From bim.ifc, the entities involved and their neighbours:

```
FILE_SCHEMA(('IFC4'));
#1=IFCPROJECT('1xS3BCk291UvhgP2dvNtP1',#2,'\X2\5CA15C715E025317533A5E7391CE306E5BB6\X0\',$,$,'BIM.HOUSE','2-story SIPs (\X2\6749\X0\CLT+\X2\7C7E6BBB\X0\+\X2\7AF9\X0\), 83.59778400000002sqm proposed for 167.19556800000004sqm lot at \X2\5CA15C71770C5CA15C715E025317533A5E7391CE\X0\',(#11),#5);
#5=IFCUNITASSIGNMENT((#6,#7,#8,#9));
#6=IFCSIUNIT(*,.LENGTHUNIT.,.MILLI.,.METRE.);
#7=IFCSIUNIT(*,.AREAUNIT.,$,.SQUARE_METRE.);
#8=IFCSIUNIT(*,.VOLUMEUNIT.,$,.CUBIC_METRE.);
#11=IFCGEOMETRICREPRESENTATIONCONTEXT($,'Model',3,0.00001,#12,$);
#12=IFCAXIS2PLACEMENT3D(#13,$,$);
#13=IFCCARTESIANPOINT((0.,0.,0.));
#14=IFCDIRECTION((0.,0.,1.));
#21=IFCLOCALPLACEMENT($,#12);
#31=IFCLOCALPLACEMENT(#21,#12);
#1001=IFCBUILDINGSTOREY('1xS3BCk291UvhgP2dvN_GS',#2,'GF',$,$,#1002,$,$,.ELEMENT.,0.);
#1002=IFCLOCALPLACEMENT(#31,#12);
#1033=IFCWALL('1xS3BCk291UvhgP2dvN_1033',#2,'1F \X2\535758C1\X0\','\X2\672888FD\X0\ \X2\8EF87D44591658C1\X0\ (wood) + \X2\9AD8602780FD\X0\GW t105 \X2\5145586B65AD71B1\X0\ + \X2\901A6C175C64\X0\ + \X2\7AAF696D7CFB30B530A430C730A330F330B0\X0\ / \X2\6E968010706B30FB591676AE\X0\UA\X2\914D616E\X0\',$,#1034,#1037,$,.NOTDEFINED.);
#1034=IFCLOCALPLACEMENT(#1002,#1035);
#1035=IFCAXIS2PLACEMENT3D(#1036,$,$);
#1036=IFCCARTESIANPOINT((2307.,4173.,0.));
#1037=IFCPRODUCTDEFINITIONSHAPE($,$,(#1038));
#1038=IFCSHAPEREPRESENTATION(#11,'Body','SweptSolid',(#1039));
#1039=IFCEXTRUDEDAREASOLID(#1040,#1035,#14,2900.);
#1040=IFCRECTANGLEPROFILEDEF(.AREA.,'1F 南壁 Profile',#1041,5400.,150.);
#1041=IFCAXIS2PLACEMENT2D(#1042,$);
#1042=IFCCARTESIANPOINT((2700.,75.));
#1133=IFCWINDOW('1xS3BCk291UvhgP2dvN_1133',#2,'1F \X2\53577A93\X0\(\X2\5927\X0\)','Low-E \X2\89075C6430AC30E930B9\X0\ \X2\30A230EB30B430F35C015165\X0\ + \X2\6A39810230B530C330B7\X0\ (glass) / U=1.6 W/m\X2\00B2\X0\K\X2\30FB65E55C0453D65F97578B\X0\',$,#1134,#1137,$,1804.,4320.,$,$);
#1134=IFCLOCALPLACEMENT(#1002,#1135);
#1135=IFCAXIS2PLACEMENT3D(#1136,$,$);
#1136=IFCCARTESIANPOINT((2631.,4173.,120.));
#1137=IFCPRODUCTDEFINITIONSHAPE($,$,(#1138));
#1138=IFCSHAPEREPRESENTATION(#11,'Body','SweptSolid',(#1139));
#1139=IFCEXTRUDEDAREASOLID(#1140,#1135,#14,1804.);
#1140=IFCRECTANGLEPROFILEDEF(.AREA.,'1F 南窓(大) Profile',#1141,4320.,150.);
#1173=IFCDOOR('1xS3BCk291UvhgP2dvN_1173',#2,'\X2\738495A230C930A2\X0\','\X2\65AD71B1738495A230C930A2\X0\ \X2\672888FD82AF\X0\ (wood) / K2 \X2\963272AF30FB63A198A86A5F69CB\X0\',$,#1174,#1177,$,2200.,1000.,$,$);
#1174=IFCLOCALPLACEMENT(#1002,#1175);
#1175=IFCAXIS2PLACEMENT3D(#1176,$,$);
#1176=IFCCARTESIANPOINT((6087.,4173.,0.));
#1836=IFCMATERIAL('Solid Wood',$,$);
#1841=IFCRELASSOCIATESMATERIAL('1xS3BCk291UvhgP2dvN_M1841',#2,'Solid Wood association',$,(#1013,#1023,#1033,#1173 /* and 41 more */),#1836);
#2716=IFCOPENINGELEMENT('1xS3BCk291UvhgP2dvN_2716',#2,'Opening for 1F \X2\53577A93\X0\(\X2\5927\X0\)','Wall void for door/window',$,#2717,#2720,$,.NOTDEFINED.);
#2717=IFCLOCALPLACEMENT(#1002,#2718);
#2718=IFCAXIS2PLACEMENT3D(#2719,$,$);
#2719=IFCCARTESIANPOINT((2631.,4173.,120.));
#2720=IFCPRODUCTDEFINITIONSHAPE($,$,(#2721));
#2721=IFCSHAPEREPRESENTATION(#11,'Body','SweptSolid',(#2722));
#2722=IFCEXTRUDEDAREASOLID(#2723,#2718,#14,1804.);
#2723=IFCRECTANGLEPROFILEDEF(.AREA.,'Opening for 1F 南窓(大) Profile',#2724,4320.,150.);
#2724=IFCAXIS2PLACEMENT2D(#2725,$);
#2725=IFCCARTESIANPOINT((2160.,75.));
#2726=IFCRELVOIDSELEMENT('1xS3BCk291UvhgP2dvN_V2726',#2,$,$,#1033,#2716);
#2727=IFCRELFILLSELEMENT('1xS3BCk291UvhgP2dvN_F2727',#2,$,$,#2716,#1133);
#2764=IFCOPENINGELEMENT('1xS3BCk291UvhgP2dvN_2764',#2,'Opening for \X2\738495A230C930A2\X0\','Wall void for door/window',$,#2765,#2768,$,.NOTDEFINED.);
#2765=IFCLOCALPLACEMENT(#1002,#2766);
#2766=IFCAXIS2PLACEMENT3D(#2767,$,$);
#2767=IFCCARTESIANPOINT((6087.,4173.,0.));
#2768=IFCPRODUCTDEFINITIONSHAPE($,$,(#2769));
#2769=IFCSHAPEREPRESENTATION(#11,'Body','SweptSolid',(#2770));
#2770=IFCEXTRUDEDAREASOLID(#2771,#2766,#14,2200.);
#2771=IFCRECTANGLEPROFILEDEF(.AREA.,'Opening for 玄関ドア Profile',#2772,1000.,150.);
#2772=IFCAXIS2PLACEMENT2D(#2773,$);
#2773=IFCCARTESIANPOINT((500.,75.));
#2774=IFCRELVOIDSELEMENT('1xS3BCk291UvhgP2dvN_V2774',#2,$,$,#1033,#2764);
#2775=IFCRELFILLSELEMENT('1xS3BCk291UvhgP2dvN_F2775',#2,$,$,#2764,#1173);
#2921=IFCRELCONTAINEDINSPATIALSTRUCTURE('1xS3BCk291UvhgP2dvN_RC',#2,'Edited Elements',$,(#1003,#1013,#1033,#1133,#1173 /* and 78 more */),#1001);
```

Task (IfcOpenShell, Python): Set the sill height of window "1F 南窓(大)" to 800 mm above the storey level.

```python
import numpy as np
import ifcopenshell
import ifcopenshell.api.geometry
import ifcopenshell.geom
import ifcopenshell.util.element
import ifcopenshell.util.placement
import ifcopenshell.util.shape
import ifcopenshell.util.unit

model = ifcopenshell.open("bim.ifc")
unit_scale = ifcopenshell.util.unit.calculate_unit_scale(model)

window = model.by_guid("1xS3BCk291UvhgP2dvN_1133")
opening = window.FillsVoids[0].RelatingOpeningElement
storey = ifcopenshell.util.element.get_container(window, ifc_class="IfcBuildingStorey")
level = ifcopenshell.util.placement.get_local_placement(storey.ObjectPlacement)[2, 3]

# The opening's origin need not be at the sill, so measure its lowest point.
shape = ifcopenshell.geom.create_shape(ifcopenshell.geom.settings(), opening)
bottom = ifcopenshell.util.shape.get_shape_bottom_elevation(shape, shape.geometry) / unit_scale
dz = level + 800.0 - bottom

shift = np.array([0.0, 0.0, dz])
# The window is not placed relative to its opening, so move both.
for product in (opening, window):
    matrix = ifcopenshell.util.placement.get_local_placement(product.ObjectPlacement)
    matrix[:3, 3] += shift
    ifcopenshell.api.geometry.edit_object_placement(model, product=product, matrix=matrix, is_si=False)

print(f"moved by {dz * unit_scale:+.3f} m")

model.write("bim-out.ifc")
```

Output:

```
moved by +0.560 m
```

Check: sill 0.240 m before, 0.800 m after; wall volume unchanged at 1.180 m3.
